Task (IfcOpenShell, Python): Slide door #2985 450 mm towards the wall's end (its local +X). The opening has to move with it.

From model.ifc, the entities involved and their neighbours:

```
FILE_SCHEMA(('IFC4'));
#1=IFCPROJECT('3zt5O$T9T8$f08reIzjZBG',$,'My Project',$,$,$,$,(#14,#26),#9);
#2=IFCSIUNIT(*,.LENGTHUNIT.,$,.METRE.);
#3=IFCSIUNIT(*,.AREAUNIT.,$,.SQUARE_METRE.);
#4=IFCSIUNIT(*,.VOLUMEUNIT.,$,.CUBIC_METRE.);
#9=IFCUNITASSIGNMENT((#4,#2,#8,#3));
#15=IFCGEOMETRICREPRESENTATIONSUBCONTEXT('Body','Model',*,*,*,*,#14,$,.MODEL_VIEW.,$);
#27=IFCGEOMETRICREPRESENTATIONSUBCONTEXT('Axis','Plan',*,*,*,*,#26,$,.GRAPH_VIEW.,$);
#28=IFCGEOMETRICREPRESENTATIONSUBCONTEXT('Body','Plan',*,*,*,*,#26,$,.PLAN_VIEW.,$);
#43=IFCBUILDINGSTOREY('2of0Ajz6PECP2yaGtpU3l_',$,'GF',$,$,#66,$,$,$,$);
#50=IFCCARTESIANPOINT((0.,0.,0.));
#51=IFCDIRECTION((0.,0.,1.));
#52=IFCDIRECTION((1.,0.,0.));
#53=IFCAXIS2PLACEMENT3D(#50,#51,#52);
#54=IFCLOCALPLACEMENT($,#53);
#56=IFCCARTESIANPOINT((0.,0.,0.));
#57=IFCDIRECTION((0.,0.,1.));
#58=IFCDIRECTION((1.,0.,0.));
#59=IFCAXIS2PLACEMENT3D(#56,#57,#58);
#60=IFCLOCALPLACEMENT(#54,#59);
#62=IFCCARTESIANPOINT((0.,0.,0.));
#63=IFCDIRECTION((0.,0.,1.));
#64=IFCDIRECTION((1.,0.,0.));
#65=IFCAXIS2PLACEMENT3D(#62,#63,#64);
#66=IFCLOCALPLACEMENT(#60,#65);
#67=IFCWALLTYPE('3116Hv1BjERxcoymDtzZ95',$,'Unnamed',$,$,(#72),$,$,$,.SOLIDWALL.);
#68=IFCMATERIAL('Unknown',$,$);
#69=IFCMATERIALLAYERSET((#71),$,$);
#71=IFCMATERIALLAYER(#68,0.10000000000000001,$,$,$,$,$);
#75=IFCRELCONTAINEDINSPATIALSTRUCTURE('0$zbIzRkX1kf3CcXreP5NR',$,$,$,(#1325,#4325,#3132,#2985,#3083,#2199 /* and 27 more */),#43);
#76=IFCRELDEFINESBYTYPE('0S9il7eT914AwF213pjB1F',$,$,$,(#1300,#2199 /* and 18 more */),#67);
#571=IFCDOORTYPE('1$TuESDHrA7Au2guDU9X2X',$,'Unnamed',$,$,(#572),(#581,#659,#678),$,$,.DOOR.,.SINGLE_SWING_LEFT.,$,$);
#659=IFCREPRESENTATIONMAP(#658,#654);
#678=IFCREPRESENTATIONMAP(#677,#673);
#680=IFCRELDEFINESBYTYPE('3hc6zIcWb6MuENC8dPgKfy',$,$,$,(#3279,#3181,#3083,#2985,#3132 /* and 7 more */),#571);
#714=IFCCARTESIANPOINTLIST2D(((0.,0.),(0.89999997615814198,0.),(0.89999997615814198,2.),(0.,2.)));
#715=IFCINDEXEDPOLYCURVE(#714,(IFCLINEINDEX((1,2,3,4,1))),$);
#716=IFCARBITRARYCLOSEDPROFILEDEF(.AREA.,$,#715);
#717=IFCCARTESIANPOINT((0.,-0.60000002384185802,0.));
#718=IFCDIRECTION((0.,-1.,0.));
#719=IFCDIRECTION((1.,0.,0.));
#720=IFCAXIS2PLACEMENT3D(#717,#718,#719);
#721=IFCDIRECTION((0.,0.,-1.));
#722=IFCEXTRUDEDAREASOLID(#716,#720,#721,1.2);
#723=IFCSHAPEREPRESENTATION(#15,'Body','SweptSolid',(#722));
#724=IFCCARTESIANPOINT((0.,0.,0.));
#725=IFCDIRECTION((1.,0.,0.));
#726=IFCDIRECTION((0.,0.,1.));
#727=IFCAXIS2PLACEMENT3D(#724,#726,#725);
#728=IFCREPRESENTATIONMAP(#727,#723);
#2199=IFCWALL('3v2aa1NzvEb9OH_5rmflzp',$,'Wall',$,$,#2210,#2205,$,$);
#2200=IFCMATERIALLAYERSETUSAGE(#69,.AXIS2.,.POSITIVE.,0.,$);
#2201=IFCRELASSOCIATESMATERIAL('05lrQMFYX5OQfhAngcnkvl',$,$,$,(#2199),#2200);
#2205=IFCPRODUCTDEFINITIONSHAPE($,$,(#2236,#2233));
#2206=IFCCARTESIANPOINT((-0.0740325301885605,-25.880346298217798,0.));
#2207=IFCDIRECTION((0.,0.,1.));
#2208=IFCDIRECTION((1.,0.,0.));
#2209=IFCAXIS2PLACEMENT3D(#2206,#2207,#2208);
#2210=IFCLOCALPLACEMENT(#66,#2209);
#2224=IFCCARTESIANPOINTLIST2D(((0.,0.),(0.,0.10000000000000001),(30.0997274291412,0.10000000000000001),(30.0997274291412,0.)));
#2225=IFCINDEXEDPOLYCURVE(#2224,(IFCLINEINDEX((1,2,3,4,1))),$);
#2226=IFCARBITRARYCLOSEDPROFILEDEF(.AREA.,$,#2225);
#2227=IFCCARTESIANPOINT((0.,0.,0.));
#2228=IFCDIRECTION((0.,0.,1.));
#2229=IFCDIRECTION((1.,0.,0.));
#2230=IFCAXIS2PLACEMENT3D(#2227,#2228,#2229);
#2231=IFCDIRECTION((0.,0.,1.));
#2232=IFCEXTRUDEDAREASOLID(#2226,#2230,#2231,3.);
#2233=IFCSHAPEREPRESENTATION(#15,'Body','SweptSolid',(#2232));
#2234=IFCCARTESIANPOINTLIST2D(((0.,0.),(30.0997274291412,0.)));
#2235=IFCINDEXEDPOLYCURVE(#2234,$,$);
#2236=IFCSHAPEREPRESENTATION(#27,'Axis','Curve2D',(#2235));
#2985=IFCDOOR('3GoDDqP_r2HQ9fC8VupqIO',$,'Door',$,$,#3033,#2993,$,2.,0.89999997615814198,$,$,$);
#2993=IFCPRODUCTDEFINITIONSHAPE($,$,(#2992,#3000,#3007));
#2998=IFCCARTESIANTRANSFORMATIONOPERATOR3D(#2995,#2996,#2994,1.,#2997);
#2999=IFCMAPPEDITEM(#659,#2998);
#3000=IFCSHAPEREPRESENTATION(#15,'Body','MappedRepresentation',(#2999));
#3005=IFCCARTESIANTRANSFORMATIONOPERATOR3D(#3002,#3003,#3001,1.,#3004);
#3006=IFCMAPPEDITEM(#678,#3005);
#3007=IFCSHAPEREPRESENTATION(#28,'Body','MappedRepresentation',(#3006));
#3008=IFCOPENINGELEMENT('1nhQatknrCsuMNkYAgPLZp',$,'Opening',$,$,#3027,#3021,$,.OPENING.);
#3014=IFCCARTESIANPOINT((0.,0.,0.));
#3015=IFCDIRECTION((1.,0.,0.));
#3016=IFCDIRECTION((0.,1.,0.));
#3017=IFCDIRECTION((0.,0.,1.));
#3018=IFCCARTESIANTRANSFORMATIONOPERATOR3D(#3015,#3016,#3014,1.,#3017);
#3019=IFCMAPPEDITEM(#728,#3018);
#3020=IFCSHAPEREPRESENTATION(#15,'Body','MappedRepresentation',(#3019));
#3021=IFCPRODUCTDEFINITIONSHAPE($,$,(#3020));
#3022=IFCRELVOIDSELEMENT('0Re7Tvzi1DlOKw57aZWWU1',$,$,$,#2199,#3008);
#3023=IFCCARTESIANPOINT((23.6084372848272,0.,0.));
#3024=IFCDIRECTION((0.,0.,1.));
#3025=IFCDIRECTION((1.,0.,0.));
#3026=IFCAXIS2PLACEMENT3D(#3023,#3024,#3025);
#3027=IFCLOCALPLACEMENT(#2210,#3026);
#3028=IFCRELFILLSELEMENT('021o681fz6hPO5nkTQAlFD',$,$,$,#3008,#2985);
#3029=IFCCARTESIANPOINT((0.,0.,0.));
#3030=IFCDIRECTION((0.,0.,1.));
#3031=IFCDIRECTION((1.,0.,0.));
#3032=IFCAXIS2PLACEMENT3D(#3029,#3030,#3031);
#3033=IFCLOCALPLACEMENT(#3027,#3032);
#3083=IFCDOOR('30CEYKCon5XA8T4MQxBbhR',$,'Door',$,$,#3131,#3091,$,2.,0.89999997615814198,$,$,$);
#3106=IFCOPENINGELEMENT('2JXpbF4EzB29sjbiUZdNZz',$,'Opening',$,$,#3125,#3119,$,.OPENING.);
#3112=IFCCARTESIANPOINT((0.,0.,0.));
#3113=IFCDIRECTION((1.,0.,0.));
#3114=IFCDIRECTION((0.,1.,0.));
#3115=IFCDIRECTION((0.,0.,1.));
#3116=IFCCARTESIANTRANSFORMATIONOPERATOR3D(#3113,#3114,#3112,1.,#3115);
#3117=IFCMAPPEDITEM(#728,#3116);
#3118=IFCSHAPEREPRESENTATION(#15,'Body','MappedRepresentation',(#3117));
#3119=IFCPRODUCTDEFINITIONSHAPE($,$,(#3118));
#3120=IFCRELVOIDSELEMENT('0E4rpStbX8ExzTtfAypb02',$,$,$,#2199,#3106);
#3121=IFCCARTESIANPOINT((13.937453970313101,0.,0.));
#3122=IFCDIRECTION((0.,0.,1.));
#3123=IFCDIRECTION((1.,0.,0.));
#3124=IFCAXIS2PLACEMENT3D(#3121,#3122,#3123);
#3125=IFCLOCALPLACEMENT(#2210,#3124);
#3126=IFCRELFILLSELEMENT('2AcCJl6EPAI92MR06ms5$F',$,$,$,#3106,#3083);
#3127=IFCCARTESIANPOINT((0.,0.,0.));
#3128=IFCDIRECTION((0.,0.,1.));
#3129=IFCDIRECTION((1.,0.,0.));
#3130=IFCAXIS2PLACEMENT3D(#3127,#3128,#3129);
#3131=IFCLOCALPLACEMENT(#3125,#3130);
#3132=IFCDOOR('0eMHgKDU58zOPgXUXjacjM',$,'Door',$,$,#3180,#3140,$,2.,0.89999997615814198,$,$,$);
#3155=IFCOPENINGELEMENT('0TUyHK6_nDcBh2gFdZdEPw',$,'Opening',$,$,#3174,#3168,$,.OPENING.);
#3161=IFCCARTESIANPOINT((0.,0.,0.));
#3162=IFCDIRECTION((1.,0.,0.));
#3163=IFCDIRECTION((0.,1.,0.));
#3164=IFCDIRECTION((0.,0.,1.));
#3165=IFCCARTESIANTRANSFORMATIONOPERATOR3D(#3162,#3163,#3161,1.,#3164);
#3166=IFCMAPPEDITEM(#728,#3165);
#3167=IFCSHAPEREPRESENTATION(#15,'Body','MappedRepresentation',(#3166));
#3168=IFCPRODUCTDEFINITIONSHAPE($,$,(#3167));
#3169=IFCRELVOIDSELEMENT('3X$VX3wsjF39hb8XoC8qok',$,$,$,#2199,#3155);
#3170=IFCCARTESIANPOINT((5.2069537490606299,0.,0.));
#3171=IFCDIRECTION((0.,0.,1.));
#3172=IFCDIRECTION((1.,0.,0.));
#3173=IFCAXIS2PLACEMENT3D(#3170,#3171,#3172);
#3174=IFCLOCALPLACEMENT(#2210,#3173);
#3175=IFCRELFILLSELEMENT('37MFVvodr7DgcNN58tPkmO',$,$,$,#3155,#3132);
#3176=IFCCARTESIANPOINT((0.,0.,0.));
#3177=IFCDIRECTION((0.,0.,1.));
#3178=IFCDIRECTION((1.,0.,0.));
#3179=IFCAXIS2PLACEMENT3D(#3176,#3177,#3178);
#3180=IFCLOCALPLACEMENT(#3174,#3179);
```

```python
import ifcopenshell
import ifcopenshell.api.geometry
import ifcopenshell.util.placement
import ifcopenshell.util.unit

model = ifcopenshell.open("model.ifc")
unit_scale = ifcopenshell.util.unit.calculate_unit_scale(model)

door = model.by_guid("3GoDDqP_r2HQ9fC8VupqIO")
opening = door.FillsVoids[0].RelatingOpeningElement
wall = opening.VoidsElements[0].RelatingBuildingElement

wall_matrix = ifcopenshell.util.placement.get_local_placement(wall.ObjectPlacement)
shift = wall_matrix[:3, 0] * 0.45 / unit_scale
before = ifcopenshell.util.placement.get_local_placement(door.ObjectPlacement)[:3, 3].copy()

# The door is placed relative to its opening, so it follows when the opening moves.
matrix = ifcopenshell.util.placement.get_local_placement(opening.ObjectPlacement)
matrix[:3, 3] += shift
ifcopenshell.api.geometry.edit_object_placement(
    model, product=opening, matrix=matrix, is_si=False, should_transform_children=True
)

after = ifcopenshell.util.placement.get_local_placement(door.ObjectPlacement)[:3, 3]
print("door moved by", (after - before).round(3) + 0.0)

model.write("model_rev.ifc")
```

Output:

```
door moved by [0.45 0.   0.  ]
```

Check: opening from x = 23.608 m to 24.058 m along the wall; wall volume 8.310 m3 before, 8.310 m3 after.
